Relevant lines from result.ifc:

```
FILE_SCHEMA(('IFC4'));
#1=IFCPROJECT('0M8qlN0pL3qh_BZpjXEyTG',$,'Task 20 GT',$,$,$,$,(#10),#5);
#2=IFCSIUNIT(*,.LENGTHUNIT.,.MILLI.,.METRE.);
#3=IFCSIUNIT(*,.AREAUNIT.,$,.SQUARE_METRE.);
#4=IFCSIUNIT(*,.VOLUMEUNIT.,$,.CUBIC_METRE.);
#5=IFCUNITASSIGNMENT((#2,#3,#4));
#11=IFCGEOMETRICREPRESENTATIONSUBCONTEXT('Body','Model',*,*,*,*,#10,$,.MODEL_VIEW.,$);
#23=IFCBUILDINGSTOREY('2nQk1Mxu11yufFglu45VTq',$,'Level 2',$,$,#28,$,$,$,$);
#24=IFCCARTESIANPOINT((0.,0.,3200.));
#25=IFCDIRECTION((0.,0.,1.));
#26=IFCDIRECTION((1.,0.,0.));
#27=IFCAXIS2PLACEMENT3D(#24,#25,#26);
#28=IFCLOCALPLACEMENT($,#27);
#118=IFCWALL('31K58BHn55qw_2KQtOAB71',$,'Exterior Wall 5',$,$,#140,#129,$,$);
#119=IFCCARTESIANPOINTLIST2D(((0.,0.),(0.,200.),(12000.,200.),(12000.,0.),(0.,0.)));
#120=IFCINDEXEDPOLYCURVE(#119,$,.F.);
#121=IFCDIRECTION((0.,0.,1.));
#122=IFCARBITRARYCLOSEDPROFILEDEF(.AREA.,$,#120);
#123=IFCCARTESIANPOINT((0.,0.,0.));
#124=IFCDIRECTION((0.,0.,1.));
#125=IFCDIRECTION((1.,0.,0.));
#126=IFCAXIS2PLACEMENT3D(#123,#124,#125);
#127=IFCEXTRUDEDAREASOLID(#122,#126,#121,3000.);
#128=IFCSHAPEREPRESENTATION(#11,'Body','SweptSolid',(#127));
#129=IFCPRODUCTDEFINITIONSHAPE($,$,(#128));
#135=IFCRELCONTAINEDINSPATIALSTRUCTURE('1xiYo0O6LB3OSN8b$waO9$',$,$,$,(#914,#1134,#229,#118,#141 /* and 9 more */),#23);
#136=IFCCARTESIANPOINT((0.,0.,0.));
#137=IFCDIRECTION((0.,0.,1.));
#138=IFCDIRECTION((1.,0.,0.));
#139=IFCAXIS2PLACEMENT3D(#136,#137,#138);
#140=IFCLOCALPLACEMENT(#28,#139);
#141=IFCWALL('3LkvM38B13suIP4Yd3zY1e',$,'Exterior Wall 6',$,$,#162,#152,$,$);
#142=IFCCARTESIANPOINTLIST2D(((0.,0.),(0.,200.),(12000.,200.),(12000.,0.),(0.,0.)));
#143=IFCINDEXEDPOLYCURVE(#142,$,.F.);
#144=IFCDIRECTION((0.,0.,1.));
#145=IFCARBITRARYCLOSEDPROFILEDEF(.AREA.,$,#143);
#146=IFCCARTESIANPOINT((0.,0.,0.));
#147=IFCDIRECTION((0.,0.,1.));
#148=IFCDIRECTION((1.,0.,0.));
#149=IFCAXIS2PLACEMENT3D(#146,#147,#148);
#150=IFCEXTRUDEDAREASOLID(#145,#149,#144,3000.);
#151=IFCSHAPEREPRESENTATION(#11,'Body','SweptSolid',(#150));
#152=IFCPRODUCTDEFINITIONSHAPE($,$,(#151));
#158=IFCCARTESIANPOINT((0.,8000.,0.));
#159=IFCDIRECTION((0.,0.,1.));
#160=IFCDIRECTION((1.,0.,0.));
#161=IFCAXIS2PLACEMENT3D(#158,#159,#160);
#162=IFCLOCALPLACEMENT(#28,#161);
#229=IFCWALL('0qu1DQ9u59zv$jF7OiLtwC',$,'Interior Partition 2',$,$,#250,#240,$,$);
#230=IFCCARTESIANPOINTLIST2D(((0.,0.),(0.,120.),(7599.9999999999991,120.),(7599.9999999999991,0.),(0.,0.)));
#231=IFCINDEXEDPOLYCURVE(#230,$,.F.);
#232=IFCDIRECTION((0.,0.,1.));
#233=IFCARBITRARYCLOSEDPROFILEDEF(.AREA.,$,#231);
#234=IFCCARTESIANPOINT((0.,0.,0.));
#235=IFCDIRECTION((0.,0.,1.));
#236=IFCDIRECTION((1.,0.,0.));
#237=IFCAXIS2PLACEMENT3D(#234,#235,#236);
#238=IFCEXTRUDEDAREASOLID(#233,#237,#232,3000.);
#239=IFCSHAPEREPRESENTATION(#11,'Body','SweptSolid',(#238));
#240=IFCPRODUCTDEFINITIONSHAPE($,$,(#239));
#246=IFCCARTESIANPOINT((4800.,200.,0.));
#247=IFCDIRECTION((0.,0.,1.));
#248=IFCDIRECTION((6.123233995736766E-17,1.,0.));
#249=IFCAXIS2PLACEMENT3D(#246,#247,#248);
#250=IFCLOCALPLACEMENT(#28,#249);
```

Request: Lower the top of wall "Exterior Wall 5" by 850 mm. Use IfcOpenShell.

```python
import ifcopenshell
import ifcopenshell.geom
import ifcopenshell.util.representation
import ifcopenshell.util.shape

model = ifcopenshell.open("result.ifc")
settings = ifcopenshell.geom.settings()


def volume(element):
    """Net volume in cubic metres, openings subtracted."""
    shape = ifcopenshell.geom.create_shape(settings, element)
    return ifcopenshell.util.shape.get_volume(shape.geometry)


wall = model.by_guid("31K58BHn55qw_2KQtOAB71")
before = volume(wall)

body = ifcopenshell.util.representation.get_representation(wall, "Model", "Body")
solid = body.Items[0]
old_height = solid.Depth
solid.Depth -= 850.0
after = volume(wall)

print(f"height {old_height:g} -> {solid.Depth:g}, volume {before:.3f} -> {after:.3f} m3")

model.write("result_v2.ifc")
```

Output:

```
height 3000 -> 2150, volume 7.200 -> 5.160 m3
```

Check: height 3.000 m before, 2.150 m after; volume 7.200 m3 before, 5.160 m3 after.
